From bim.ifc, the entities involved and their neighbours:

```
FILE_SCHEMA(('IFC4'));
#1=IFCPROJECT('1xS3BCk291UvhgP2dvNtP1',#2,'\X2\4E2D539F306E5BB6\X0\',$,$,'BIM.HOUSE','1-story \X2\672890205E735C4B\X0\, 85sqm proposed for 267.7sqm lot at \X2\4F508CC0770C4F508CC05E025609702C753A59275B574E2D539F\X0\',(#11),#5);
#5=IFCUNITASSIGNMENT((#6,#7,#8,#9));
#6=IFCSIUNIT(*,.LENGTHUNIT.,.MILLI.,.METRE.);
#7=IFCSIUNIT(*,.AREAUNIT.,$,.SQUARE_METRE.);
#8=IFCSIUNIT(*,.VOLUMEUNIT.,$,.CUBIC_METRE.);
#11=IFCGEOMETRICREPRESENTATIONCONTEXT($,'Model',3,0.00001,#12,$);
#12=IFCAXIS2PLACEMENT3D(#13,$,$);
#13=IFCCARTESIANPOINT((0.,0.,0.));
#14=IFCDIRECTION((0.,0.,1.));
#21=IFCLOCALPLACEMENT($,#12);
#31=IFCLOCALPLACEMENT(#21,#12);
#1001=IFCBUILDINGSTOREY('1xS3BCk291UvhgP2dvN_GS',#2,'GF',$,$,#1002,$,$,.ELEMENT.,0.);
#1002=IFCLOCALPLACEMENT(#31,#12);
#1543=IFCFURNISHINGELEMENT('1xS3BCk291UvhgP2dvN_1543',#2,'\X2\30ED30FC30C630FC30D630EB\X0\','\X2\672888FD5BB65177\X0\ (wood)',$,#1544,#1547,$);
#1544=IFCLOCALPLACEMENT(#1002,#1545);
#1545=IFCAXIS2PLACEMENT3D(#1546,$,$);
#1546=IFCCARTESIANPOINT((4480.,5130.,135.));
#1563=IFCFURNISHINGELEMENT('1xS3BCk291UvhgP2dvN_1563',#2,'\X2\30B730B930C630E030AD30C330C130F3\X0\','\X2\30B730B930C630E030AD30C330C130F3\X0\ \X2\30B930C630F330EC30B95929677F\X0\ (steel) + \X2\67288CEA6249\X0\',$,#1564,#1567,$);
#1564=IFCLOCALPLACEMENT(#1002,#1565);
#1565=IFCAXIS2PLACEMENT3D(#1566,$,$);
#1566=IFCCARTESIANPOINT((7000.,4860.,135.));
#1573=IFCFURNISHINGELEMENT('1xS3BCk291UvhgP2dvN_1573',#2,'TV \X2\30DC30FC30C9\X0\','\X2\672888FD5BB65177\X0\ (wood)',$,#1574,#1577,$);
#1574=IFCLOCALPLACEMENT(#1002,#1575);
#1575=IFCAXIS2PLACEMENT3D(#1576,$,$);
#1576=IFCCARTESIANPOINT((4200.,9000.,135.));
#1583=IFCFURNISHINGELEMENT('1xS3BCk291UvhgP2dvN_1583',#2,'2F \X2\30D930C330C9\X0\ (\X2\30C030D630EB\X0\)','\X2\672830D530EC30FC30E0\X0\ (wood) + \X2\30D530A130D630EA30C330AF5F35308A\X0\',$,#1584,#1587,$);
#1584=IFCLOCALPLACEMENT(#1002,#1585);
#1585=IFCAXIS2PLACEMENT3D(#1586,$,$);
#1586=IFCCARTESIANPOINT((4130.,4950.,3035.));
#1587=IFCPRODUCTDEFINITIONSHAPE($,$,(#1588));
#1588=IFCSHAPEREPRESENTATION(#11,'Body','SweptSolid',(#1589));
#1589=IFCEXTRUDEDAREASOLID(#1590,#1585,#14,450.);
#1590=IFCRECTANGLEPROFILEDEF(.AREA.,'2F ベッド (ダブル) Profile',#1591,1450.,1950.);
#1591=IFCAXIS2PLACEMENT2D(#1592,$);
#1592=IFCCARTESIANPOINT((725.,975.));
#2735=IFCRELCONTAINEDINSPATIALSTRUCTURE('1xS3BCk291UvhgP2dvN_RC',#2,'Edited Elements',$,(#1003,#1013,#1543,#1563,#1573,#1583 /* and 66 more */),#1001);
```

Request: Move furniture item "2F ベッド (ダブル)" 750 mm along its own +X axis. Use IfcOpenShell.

```python
import ifcopenshell
import ifcopenshell.api.geometry
import ifcopenshell.util.placement
import ifcopenshell.util.unit

model = ifcopenshell.open("bim.ifc")
unit_scale = ifcopenshell.util.unit.calculate_unit_scale(model)

item = model.by_guid("1xS3BCk291UvhgP2dvN_1583")
matrix = ifcopenshell.util.placement.get_local_placement(item.ObjectPlacement)
matrix[:3, 3] += matrix[:3, 0] * 0.75 / unit_scale
ifcopenshell.api.geometry.edit_object_placement(model, product=item, matrix=matrix, is_si=False)

print(ifcopenshell.util.placement.get_local_placement(item.ObjectPlacement).round(3) + 0.0)

model.write("bim_rev.ifc")
```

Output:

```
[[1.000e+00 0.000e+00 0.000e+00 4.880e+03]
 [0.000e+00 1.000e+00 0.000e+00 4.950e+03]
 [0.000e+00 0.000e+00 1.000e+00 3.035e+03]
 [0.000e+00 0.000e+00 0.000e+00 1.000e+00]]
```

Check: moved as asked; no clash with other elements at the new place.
